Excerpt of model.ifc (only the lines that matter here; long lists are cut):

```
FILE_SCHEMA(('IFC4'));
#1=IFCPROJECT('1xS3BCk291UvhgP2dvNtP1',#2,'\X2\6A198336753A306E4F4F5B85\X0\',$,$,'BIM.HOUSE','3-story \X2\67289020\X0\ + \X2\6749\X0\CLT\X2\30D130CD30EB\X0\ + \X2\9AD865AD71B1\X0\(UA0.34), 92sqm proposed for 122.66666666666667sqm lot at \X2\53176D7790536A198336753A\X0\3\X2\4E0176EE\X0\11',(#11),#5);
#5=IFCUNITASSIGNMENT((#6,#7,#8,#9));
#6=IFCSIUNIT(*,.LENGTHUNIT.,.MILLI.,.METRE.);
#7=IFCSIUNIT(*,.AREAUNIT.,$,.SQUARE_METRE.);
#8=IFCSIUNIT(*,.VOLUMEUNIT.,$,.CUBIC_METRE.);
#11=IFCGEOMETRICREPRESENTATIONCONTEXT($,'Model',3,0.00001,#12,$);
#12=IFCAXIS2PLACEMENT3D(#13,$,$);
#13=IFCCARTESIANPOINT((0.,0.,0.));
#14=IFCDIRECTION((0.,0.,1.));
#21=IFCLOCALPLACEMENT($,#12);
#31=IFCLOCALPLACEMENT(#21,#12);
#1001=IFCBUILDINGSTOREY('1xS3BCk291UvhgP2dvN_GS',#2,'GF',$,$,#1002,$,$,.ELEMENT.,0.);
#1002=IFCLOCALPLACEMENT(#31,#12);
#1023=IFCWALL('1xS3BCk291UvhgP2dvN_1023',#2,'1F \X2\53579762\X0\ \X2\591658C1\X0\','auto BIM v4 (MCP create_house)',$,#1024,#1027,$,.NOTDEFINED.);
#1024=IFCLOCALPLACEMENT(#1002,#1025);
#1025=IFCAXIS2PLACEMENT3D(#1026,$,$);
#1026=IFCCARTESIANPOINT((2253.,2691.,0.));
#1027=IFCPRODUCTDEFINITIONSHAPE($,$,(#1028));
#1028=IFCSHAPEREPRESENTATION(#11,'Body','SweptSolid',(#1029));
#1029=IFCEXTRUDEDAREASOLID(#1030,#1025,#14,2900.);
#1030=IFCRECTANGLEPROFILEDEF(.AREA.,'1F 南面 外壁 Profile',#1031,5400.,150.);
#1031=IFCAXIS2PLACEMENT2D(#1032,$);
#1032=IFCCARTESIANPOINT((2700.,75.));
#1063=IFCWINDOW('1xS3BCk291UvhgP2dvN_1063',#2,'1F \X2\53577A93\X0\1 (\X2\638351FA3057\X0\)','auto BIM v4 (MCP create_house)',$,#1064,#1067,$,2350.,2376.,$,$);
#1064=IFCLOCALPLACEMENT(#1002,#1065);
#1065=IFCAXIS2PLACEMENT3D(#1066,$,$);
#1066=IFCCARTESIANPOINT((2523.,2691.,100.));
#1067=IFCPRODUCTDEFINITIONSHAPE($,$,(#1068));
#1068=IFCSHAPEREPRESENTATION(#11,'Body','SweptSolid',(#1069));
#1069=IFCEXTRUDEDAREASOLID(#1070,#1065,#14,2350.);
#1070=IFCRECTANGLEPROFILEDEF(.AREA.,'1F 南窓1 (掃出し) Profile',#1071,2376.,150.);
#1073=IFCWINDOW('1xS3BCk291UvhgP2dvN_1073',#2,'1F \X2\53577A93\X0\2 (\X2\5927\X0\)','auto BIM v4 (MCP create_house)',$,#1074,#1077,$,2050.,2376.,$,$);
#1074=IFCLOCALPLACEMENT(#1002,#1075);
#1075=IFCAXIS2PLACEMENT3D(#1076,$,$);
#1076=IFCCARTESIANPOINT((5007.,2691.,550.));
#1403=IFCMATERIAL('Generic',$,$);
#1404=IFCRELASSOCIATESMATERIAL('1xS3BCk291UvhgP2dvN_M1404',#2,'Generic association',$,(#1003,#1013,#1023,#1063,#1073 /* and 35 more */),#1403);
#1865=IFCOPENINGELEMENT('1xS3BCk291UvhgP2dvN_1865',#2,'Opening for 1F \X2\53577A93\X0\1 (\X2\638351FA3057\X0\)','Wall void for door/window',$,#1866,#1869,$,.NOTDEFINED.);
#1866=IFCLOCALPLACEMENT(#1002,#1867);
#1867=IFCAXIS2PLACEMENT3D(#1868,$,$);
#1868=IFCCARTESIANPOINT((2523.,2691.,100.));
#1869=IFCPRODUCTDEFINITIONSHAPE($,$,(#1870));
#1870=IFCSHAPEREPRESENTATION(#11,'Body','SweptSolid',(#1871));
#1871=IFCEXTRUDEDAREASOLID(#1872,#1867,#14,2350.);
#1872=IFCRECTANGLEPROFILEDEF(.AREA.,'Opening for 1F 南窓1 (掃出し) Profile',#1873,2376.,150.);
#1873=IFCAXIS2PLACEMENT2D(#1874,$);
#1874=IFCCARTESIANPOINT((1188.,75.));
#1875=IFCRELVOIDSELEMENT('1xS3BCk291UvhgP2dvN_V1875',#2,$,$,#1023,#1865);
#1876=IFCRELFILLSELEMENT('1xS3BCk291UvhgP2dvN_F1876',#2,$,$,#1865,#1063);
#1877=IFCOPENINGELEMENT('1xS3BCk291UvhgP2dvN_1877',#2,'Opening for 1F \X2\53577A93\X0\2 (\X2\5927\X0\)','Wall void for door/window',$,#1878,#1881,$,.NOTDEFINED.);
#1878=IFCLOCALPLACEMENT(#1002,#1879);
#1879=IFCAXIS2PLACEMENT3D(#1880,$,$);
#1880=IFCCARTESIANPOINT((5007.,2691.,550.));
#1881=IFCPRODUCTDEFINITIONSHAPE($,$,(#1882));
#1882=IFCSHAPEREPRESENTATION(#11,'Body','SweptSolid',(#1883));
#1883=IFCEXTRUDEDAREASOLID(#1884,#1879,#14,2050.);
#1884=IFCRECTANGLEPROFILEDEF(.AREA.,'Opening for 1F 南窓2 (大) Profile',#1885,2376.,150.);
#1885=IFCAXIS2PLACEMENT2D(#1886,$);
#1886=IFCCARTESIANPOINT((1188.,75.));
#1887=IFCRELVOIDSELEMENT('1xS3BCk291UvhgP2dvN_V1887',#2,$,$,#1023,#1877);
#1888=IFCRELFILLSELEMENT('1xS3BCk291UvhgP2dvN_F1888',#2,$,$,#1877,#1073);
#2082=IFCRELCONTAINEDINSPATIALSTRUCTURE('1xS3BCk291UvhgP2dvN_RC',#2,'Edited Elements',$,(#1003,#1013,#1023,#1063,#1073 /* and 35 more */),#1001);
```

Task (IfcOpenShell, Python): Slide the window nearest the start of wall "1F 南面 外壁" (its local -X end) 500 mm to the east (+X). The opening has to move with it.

```python
import ifcopenshell
import ifcopenshell.api.geometry
import ifcopenshell.util.placement

model = ifcopenshell.open("model.ifc")

window = model.by_guid("1xS3BCk291UvhgP2dvN_1063")
opening = window.FillsVoids[0].RelatingOpeningElement
wall = opening.VoidsElements[0].RelatingBuildingElement

wall_matrix = ifcopenshell.util.placement.get_local_placement(wall.ObjectPlacement)
shift = wall_matrix[:3, 0] * 500.0
before = ifcopenshell.util.placement.get_local_placement(window.ObjectPlacement)[:3, 3].copy()

# The window is not placed relative to its opening, so move both.
for product in (opening, window):
    matrix = ifcopenshell.util.placement.get_local_placement(product.ObjectPlacement)
    matrix[:3, 3] += shift
    ifcopenshell.api.geometry.edit_object_placement(model, product=product, matrix=matrix, is_si=False)

after = ifcopenshell.util.placement.get_local_placement(window.ObjectPlacement)[:3, 3]
print("window moved by", (after - before).round(3) + 0.0)

model.write("model_updated.ifc")
```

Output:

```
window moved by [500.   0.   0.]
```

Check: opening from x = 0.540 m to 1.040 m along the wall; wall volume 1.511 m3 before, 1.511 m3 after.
